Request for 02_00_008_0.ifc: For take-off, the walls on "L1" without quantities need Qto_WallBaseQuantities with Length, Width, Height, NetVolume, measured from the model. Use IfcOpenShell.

First a look at what the model holds.

```python
import ifcopenshell
import ifcopenshell.util.element
import ifcopenshell.util.unit

model = ifcopenshell.open("02_00_008_0.ifc")
print(model.schema)
for unit_type in ("LENGTHUNIT", "AREAUNIT", "VOLUMEUNIT"):
    print(unit_type, ifcopenshell.util.unit.calculate_unit_scale(model, unit_type))
storey = next(s for s in model.by_type("IfcBuildingStorey") if s.Name == "L1")
walls = [e for e in ifcopenshell.util.element.get_decomposition(storey) if e.is_a("IfcWall")]
for e in sorted(walls, key=lambda e: e.id()):
    print(e.id(), e.is_a(), e.Name, list(ifcopenshell.util.element.get_psets(e, qtos_only=True)), sep=" | ")
```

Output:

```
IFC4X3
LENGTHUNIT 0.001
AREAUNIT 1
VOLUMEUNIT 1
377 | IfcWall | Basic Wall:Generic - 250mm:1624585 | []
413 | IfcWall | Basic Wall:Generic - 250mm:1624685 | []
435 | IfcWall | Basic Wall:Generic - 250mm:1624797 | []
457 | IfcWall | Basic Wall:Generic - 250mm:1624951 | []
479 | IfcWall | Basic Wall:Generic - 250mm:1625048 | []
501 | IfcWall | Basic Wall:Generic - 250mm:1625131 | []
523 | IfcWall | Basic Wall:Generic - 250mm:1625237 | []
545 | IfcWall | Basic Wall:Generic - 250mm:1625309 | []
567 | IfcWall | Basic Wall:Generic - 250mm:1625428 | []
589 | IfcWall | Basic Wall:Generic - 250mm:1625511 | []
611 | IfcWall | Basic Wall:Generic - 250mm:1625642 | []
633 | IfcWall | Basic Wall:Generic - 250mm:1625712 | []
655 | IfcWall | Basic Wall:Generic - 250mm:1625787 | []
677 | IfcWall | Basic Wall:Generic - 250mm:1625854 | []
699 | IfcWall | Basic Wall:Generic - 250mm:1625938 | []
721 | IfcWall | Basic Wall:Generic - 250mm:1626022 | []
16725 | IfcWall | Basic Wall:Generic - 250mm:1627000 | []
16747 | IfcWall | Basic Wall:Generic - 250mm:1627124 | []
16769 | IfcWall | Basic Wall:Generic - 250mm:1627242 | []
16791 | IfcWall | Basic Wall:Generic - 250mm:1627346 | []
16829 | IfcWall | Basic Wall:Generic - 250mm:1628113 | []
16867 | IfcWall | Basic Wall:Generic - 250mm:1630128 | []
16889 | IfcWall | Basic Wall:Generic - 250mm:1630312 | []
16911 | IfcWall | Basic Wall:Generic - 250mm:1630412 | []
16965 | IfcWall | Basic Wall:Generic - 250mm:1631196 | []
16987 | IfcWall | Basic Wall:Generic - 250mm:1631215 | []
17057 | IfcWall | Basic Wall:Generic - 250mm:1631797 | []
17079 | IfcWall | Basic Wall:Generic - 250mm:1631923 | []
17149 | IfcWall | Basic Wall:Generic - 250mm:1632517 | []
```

```python
import ifcopenshell
import ifcopenshell.api.pset
import ifcopenshell.geom
import ifcopenshell.util.element
import ifcopenshell.util.shape
import ifcopenshell.util.unit

model = ifcopenshell.open("02_00_008_0.ifc")
unit_scale = ifcopenshell.util.unit.calculate_unit_scale(model)
volume_scale = ifcopenshell.util.unit.calculate_unit_scale(model, "VOLUMEUNIT")
settings = ifcopenshell.geom.settings()

storey = next(s for s in model.by_type("IfcBuildingStorey") if s.Name == "L1")
walls = [e for e in ifcopenshell.util.element.get_decomposition(storey) if e.is_a("IfcWall")]

for e in sorted(walls, key=lambda e: e.id()):
    if ifcopenshell.util.element.get_psets(e, qtos_only=True, should_inherit=False):
        continue
    # Geometry comes back in metres, in the element's own axes.
    shape = ifcopenshell.geom.create_shape(settings, e)
    values = {
        "Length": ifcopenshell.util.shape.get_x(shape.geometry) / unit_scale,
        "Width": ifcopenshell.util.shape.get_y(shape.geometry) / unit_scale,
        "Height": ifcopenshell.util.shape.get_z(shape.geometry) / unit_scale,
        "NetVolume": ifcopenshell.util.shape.get_volume(shape.geometry) / volume_scale,
    }
    qto = ifcopenshell.api.pset.add_qto(model, product=e, name="Qto_WallBaseQuantities")
    ifcopenshell.api.pset.edit_qto(model, qto=qto, properties=values)
    print(e.id(), {k: round(v, 3) for k, v in values.items()})

model.write("02_00_008_0_edited.ifc")
```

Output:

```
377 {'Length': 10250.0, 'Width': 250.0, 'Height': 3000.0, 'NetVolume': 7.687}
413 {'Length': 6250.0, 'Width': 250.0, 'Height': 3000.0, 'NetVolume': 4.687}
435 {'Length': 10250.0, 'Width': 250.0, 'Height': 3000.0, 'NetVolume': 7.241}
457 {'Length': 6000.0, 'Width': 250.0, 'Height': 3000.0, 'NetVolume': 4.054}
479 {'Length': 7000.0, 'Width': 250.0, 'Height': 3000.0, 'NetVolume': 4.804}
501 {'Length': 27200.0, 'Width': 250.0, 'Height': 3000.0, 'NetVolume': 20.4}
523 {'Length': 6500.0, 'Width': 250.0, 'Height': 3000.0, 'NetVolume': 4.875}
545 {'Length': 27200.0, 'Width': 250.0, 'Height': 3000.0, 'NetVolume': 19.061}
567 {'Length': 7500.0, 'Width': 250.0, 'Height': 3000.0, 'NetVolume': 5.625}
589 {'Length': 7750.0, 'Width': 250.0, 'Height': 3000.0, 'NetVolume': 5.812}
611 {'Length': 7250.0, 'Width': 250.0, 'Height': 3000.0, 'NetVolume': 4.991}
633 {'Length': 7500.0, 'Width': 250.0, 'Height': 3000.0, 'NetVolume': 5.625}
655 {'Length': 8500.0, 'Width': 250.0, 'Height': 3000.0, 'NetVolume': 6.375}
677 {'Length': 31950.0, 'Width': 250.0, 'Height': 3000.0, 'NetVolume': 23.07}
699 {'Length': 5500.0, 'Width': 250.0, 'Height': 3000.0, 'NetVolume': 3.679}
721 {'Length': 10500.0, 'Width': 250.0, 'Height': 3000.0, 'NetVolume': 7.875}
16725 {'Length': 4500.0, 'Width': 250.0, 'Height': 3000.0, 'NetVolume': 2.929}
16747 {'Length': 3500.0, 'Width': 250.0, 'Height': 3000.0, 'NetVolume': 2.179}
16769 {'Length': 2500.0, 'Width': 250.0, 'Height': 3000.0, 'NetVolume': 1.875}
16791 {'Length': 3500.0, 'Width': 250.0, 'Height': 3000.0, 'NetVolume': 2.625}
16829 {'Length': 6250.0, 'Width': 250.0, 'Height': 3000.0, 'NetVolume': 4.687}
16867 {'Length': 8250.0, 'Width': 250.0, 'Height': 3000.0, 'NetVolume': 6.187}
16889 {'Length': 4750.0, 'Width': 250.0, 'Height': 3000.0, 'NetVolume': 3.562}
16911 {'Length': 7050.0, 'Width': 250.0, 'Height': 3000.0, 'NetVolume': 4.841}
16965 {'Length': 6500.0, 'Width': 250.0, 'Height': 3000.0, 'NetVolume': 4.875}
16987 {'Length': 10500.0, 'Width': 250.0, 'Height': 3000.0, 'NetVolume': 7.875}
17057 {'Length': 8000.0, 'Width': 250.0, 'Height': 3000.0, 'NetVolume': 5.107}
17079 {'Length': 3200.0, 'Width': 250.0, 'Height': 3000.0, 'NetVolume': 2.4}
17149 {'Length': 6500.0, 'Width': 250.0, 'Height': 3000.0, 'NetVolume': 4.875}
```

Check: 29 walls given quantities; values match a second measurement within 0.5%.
